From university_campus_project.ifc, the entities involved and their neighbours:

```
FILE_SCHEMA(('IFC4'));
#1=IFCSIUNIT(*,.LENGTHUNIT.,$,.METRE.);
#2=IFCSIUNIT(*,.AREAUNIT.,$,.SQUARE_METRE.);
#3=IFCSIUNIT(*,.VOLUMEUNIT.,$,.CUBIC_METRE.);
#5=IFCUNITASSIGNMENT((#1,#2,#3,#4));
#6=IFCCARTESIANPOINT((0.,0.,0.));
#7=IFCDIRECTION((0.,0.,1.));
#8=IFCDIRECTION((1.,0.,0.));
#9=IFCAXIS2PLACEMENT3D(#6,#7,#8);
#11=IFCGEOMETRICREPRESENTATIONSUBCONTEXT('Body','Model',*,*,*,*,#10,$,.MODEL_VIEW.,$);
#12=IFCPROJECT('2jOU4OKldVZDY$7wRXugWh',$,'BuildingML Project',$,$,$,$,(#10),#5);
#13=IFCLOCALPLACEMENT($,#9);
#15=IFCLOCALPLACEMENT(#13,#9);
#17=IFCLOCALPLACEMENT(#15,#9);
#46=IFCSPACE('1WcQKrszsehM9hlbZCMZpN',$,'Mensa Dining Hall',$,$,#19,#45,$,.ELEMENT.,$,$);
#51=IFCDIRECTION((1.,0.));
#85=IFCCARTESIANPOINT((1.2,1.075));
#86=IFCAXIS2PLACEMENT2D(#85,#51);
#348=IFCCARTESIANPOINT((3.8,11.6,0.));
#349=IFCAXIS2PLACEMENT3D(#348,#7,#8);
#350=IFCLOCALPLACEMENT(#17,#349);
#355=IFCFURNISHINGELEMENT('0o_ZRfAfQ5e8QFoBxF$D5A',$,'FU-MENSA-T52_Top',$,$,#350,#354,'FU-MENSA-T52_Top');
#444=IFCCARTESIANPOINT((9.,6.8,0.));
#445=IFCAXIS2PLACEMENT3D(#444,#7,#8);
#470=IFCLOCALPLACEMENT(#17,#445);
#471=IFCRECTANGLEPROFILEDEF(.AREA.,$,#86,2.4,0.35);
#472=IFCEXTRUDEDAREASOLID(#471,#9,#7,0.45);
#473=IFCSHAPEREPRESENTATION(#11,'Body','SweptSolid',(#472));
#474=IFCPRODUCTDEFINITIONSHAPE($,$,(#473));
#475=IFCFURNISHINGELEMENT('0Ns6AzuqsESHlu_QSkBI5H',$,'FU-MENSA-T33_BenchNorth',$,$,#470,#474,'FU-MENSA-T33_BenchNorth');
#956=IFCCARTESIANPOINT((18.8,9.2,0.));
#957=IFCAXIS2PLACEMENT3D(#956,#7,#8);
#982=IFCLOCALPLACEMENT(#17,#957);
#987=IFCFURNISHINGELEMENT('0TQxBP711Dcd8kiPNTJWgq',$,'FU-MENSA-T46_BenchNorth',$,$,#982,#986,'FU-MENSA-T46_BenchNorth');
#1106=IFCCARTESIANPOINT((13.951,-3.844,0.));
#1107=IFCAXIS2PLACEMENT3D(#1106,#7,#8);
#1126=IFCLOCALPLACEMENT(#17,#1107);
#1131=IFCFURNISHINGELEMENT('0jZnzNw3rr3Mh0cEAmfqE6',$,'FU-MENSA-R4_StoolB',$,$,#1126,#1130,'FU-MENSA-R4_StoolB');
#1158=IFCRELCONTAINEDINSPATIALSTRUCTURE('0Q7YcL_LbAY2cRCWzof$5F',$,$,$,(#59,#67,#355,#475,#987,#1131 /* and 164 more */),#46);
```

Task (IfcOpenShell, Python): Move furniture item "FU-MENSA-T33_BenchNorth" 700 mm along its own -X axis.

```python
import ifcopenshell
import ifcopenshell.api.geometry
import ifcopenshell.util.placement
import ifcopenshell.util.unit

model = ifcopenshell.open("university_campus_project.ifc")
unit_scale = ifcopenshell.util.unit.calculate_unit_scale(model)

item = model.by_guid("0Ns6AzuqsESHlu_QSkBI5H")
matrix = ifcopenshell.util.placement.get_local_placement(item.ObjectPlacement)
matrix[:3, 3] -= matrix[:3, 0] * 0.7 / unit_scale
ifcopenshell.api.geometry.edit_object_placement(model, product=item, matrix=matrix, is_si=False)

print(ifcopenshell.util.placement.get_local_placement(item.ObjectPlacement).round(3) + 0.0)

model.write("university_campus_project_updated.ifc")
```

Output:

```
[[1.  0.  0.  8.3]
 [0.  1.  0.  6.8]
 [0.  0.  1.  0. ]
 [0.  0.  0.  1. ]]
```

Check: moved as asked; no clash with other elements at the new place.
